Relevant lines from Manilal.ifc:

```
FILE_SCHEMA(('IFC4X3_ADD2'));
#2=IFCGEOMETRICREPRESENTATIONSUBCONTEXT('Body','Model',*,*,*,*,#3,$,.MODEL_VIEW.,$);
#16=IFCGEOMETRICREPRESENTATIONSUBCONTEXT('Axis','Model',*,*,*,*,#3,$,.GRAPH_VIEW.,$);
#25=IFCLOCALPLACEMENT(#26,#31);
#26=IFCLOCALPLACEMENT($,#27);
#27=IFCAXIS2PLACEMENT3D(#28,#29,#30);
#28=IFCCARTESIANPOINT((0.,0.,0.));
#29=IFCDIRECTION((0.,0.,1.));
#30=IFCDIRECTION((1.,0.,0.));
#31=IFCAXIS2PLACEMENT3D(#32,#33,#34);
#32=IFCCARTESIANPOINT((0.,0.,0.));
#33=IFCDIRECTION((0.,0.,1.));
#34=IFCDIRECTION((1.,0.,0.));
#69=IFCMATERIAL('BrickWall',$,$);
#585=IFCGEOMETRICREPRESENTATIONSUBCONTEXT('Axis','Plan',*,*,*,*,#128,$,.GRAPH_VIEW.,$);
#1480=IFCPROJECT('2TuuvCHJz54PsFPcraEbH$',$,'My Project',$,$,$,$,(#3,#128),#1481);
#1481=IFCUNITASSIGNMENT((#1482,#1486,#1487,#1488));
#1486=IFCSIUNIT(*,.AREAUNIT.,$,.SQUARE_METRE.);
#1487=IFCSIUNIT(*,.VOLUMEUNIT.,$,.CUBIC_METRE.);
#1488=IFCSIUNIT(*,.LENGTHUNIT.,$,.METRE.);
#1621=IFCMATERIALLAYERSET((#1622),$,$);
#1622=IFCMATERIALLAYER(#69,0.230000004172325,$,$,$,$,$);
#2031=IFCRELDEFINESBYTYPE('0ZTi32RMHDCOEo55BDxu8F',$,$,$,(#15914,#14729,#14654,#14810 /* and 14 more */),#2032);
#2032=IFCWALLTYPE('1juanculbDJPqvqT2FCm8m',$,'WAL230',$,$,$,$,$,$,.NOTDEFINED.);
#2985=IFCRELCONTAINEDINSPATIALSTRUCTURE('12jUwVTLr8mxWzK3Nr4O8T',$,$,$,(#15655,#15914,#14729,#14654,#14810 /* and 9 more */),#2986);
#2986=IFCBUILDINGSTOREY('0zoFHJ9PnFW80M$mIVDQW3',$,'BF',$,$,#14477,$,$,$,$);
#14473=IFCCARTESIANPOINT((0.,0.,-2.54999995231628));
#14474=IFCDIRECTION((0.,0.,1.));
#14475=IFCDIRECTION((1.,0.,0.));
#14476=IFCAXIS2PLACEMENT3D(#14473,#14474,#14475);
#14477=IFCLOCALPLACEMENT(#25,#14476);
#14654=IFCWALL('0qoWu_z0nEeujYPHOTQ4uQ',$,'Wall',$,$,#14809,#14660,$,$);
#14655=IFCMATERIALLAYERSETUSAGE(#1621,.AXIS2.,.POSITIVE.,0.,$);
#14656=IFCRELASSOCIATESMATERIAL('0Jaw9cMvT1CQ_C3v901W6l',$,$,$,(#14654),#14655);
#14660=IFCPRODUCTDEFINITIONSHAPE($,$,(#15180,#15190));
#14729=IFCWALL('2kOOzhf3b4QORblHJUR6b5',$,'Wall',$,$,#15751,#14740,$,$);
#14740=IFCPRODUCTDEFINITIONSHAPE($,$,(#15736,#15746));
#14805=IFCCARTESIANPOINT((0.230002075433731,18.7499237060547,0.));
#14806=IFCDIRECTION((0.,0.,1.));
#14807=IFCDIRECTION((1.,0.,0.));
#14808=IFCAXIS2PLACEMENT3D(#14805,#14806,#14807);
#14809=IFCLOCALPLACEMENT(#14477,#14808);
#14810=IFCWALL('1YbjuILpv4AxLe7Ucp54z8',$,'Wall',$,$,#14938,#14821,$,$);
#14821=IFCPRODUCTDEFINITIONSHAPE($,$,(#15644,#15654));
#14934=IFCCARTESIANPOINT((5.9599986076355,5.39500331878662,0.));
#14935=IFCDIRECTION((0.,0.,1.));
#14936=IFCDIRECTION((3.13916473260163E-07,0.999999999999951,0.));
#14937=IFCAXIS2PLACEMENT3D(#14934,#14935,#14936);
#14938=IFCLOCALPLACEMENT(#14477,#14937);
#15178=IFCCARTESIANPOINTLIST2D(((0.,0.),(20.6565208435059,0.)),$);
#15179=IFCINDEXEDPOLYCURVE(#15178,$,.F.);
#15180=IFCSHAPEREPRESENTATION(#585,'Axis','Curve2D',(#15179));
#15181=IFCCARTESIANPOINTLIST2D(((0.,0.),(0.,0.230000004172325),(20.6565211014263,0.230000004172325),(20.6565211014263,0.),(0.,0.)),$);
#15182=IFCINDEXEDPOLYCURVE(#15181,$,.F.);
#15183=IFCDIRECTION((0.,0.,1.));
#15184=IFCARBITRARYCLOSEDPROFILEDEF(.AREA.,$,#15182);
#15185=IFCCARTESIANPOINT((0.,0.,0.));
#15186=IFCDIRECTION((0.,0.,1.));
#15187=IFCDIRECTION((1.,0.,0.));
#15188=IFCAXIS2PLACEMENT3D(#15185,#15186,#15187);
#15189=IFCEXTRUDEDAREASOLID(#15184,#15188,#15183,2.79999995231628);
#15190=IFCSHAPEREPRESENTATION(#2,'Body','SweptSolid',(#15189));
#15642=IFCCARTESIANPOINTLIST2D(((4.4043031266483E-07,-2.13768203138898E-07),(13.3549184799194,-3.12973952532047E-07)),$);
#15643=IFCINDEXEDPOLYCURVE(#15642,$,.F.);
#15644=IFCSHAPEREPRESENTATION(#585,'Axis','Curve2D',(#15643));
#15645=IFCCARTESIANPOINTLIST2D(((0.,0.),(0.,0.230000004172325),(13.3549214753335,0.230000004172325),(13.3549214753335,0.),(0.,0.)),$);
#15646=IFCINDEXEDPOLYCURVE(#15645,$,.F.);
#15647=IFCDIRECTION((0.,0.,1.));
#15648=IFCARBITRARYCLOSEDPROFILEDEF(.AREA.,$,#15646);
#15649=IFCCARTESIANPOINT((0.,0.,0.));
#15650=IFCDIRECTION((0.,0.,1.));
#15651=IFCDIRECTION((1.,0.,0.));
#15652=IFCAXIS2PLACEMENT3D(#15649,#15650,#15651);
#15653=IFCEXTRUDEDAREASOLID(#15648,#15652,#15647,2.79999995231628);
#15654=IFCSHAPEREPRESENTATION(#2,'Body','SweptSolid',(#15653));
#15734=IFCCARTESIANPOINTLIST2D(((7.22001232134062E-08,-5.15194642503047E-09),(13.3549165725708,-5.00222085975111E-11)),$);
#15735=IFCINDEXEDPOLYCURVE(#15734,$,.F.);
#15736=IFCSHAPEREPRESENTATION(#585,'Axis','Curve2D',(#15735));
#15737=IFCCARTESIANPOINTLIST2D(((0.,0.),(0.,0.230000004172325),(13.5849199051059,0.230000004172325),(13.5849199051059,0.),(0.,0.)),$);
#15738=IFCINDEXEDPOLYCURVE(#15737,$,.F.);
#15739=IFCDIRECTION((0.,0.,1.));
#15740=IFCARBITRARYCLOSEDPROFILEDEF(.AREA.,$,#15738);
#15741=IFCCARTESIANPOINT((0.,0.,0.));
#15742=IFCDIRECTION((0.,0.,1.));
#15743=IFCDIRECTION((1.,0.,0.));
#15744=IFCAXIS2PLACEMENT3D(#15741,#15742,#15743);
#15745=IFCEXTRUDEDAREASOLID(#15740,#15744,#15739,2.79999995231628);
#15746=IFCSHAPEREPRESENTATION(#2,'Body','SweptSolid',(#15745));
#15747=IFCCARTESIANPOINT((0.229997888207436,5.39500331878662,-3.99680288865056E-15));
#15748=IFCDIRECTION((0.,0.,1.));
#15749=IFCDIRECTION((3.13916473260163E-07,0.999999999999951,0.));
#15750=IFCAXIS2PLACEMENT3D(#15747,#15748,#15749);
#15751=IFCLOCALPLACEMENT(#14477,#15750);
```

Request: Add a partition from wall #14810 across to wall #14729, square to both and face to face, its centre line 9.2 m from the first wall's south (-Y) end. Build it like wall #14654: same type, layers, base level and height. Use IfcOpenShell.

```python
import numpy as np
import ifcopenshell
import ifcopenshell.api.geometry
import ifcopenshell.api.material
import ifcopenshell.api.pset
import ifcopenshell.api.root
import ifcopenshell.api.spatial
import ifcopenshell.api.type
import ifcopenshell.geom
import ifcopenshell.util.element
import ifcopenshell.util.placement
import ifcopenshell.util.representation
import ifcopenshell.util.shape
import ifcopenshell.util.unit

model = ifcopenshell.open("Manilal.ifc")
unit_scale = ifcopenshell.util.unit.calculate_unit_scale(model)
settings = ifcopenshell.geom.settings()
settings.set("use-world-coords", True)

start_wall = model.by_guid("1YbjuILpv4AxLe7Ucp54z8")
end_wall = model.by_guid("2kOOzhf3b4QORblHJUR6b5")
like = model.by_id(14654)
matrix = ifcopenshell.util.placement.get_local_placement(start_wall.ObjectPlacement)
matrix[:3, 3] *= unit_scale


def extent(element):
    """Bounding box in the first wall's axes, in metres."""
    shape = ifcopenshell.geom.create_shape(settings, element)
    points = (ifcopenshell.util.shape.get_vertices(shape.geometry) - matrix[:3, 3]) @ matrix[:3, :3]
    return points.min(axis=0), points.max(axis=0)


y_start = extent(start_wall)[1][1]
y_end = extent(end_wall)[0][1]
like_min, like_max = extent(like)
length, height = float(abs(y_end - y_start)), float(like_max[2] - like_min[2])
layer_set = ifcopenshell.util.element.get_material(like, should_skip_usage=True)
thickness = sum(layer.LayerThickness for layer in layer_set.MaterialLayers) * unit_scale

wall = ifcopenshell.api.root.create_entity(model, ifc_class="IfcWall", name="New partition")
storey = ifcopenshell.util.element.get_container(like)
ifcopenshell.api.spatial.assign_container(model, products=[wall], relating_structure=storey)
ifcopenshell.api.type.assign_type(
    model, related_objects=[wall], relating_type=ifcopenshell.util.element.get_type(like), should_map_representations=False
)
rel = ifcopenshell.api.material.assign_material(
    model, products=[wall], type="IfcMaterialLayerSetUsage", material=layer_set
)
rel.RelatingMaterial.OffsetFromReferenceLine = -thickness / 2 / unit_scale
pset = ifcopenshell.api.pset.add_pset(model, product=wall, name="Pset_WallCommon")
ifcopenshell.api.pset.edit_pset(model, pset=pset, properties={"IsExternal": False, "LoadBearing": False})

# The axis runs down the middle of the wall.
axis = ifcopenshell.api.geometry.add_axis_representation(
    model, context=ifcopenshell.util.representation.get_context(model, "Model", "Axis"), axis=[(0.0, 0.0), (length, 0.0)]
)
body = ifcopenshell.api.geometry.add_wall_representation(
    model,
    context=ifcopenshell.util.representation.get_context(model, "Model", "Body", "MODEL_VIEW"),
    length=length,
    height=height,
    thickness=thickness,
    offset=-thickness / 2,
)
for representation in (axis, body):
    ifcopenshell.api.geometry.assign_representation(model, product=wall, representation=representation)

placement = matrix @ ifcopenshell.util.placement.rotation(90, "Z")
placement[:, 3] = matrix @ np.array([extent(start_wall)[0][0] + 9.2, y_start, like_min[2], 1.0])
ifcopenshell.api.geometry.edit_object_placement(model, product=wall, matrix=placement)

print(f"partition {length:.3f} m long, {height:.3f} m high, {thickness:.3f} m thick")

model.write("Manilal-out.ifc")
```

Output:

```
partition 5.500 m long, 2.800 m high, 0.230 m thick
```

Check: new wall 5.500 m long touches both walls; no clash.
